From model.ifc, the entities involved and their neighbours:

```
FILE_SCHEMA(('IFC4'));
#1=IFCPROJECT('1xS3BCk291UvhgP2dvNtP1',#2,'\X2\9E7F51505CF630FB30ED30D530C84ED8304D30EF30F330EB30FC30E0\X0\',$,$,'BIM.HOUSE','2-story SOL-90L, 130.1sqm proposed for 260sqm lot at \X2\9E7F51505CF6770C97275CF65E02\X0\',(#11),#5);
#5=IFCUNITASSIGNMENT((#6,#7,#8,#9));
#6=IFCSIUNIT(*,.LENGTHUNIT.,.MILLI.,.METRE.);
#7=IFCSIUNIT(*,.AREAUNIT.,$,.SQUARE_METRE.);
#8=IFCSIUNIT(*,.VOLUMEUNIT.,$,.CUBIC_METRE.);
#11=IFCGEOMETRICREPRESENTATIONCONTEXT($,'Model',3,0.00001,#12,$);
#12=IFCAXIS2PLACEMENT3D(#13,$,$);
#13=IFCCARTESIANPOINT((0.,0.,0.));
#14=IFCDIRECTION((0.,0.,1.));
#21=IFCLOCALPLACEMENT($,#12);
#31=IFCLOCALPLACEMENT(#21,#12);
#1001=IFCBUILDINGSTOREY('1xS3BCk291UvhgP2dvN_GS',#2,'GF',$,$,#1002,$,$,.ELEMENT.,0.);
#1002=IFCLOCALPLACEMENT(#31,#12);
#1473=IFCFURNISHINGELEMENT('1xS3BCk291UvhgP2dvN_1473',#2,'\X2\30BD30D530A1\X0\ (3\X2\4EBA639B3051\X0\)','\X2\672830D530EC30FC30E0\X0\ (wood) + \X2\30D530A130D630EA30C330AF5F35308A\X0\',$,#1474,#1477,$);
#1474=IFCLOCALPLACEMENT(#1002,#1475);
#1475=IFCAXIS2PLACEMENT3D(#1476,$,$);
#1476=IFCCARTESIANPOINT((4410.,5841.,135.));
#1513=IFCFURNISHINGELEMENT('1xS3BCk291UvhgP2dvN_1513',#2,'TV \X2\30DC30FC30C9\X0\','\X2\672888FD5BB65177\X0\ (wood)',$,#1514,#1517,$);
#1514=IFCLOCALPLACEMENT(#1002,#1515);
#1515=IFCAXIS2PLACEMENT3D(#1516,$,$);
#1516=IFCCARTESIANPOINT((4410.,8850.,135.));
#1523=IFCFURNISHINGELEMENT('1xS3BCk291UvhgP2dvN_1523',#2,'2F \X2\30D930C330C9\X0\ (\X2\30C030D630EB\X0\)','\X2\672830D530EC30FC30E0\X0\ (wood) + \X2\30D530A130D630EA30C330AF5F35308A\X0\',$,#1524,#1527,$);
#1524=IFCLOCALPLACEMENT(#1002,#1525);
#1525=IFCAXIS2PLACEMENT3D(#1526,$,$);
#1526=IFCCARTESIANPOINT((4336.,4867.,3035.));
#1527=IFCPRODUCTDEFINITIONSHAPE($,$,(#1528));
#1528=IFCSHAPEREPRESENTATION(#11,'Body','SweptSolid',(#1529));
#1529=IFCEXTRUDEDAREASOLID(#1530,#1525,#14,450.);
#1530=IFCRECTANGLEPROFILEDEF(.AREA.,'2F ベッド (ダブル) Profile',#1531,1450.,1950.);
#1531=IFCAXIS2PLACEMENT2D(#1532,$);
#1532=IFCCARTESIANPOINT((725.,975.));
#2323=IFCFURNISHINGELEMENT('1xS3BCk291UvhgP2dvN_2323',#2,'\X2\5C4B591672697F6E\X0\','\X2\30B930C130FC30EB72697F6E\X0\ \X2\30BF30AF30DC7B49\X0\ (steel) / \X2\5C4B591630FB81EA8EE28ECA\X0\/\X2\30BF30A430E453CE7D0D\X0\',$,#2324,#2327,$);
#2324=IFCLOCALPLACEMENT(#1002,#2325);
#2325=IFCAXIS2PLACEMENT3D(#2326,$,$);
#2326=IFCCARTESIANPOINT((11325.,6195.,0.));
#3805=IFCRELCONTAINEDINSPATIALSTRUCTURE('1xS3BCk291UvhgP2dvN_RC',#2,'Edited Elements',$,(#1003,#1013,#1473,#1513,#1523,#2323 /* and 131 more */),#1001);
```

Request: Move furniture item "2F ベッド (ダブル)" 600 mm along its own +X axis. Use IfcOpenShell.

```python
import ifcopenshell
import ifcopenshell.api.geometry
import ifcopenshell.util.placement

model = ifcopenshell.open("model.ifc")

item = model.by_guid("1xS3BCk291UvhgP2dvN_1523")
matrix = ifcopenshell.util.placement.get_local_placement(item.ObjectPlacement)
matrix[:3, 3] += matrix[:3, 0] * 600.0
ifcopenshell.api.geometry.edit_object_placement(model, product=item, matrix=matrix, is_si=False)

print(ifcopenshell.util.placement.get_local_placement(item.ObjectPlacement).round(3) + 0.0)

model.write("model_updated.ifc")
```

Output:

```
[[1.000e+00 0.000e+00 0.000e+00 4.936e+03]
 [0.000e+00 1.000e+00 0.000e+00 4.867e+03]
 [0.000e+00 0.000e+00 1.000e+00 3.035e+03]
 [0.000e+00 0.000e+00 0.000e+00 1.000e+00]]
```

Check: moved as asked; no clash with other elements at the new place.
